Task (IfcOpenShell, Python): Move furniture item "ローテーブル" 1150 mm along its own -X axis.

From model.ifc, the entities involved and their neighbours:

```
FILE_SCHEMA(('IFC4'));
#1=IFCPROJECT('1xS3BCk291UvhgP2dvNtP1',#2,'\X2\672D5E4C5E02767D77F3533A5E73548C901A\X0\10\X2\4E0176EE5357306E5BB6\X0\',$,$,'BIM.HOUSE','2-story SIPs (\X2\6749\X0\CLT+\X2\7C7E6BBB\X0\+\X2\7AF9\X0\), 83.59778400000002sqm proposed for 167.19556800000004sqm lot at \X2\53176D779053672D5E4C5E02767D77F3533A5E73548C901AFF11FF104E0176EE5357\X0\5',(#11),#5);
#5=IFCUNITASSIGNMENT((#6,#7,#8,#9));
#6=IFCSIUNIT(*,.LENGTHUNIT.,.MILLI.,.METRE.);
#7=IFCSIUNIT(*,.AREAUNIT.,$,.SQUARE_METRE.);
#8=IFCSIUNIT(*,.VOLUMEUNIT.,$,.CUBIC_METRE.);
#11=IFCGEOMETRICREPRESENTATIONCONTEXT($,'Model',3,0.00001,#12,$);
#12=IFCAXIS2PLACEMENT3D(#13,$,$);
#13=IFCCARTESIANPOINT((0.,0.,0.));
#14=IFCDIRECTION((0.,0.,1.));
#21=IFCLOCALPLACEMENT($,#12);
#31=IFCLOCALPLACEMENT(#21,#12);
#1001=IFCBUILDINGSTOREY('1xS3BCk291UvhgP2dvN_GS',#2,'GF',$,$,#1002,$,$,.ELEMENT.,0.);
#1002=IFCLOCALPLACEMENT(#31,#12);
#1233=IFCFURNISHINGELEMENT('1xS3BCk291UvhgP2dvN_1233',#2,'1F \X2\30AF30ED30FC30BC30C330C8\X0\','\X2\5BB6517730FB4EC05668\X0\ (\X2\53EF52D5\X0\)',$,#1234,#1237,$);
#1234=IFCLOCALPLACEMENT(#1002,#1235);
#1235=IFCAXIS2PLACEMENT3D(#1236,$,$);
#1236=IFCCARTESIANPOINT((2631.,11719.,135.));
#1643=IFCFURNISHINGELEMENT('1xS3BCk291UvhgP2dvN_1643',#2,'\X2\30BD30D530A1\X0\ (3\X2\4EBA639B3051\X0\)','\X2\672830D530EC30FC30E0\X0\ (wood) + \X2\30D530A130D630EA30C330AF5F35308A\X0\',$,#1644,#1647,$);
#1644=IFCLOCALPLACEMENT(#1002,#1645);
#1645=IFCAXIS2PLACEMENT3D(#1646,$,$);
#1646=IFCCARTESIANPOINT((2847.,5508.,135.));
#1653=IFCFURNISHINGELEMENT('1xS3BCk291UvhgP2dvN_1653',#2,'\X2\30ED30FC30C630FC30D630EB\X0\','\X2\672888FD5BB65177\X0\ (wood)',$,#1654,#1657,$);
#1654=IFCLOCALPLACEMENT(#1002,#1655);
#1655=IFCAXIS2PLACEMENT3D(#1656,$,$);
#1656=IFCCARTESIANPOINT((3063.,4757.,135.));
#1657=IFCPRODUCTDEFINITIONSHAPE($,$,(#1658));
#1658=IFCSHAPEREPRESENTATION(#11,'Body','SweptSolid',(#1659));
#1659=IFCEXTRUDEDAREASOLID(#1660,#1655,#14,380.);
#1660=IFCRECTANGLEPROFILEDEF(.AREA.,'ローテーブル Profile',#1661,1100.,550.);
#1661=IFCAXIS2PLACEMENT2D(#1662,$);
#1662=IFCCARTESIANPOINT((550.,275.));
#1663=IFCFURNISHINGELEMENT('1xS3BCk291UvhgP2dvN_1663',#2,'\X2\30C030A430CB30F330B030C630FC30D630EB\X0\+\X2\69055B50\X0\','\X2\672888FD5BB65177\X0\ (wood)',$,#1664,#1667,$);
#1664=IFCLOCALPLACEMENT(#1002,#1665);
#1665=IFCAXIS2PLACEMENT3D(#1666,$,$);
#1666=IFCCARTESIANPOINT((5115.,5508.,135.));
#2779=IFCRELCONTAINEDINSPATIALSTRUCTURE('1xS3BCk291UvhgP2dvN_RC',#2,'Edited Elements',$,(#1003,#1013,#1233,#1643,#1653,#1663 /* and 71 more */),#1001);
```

```python
import ifcopenshell
import ifcopenshell.api.geometry
import ifcopenshell.util.placement

model = ifcopenshell.open("model.ifc")

item = model.by_guid("1xS3BCk291UvhgP2dvN_1653")
matrix = ifcopenshell.util.placement.get_local_placement(item.ObjectPlacement)
matrix[:3, 3] -= matrix[:3, 0] * 1150.0
ifcopenshell.api.geometry.edit_object_placement(model, product=item, matrix=matrix, is_si=False)

print(ifcopenshell.util.placement.get_local_placement(item.ObjectPlacement).round(3) + 0.0)

model.write("model_v2.ifc")
```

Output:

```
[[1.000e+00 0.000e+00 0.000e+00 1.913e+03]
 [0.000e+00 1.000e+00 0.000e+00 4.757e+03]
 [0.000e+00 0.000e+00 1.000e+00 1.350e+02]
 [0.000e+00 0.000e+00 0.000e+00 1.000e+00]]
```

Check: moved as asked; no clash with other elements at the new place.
